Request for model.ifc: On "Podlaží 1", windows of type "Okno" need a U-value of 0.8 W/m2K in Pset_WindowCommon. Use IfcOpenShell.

First a look at what the model holds.

```python
import ifcopenshell
import ifcopenshell.util.element

model = ifcopenshell.open("model.ifc")
print(model.schema)
storey = next(s for s in model.by_type("IfcBuildingStorey") if s.Name == "Podlaží 1")
windows = [e for e in ifcopenshell.util.element.get_decomposition(storey) if e.is_a("IfcWindow")]
seen = {}
for e in windows:
    element_type = ifcopenshell.util.element.get_type(e)
    key = (element_type.Name if element_type != e and element_type else None, ifcopenshell.util.element.get_pset(e, "Pset_WindowCommon", "ThermalTransmittance"))
    seen[key] = seen.get(key, 0) + 1
for (name, value), count in sorted(seen.items(), key=str):
    print(count, "x", name, "|", value)
```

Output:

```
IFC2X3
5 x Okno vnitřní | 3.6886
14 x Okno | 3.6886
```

```python
import ifcopenshell
import ifcopenshell.api.pset
import ifcopenshell.util.element

model = ifcopenshell.open("model.ifc")

storey = next(s for s in model.by_type("IfcBuildingStorey") if s.Name == "Podlaží 1")
windows = [e for e in ifcopenshell.util.element.get_decomposition(storey) if e.is_a("IfcWindow")]

count = 0
for e in windows:
    element_type = ifcopenshell.util.element.get_type(e)
    if element_type in (None, e) or element_type.Name != "Okno":
        continue
    # add_pset returns the element's existing set when there is one.
    pset = ifcopenshell.api.pset.add_pset(model, product=e, name="Pset_WindowCommon")
    ifcopenshell.api.pset.edit_pset(model, pset=pset, properties={"ThermalTransmittance": 0.8})
    count += 1

print(count, "windows updated")

model.write("model_rev.ifc")
```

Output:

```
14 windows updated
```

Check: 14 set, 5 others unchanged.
